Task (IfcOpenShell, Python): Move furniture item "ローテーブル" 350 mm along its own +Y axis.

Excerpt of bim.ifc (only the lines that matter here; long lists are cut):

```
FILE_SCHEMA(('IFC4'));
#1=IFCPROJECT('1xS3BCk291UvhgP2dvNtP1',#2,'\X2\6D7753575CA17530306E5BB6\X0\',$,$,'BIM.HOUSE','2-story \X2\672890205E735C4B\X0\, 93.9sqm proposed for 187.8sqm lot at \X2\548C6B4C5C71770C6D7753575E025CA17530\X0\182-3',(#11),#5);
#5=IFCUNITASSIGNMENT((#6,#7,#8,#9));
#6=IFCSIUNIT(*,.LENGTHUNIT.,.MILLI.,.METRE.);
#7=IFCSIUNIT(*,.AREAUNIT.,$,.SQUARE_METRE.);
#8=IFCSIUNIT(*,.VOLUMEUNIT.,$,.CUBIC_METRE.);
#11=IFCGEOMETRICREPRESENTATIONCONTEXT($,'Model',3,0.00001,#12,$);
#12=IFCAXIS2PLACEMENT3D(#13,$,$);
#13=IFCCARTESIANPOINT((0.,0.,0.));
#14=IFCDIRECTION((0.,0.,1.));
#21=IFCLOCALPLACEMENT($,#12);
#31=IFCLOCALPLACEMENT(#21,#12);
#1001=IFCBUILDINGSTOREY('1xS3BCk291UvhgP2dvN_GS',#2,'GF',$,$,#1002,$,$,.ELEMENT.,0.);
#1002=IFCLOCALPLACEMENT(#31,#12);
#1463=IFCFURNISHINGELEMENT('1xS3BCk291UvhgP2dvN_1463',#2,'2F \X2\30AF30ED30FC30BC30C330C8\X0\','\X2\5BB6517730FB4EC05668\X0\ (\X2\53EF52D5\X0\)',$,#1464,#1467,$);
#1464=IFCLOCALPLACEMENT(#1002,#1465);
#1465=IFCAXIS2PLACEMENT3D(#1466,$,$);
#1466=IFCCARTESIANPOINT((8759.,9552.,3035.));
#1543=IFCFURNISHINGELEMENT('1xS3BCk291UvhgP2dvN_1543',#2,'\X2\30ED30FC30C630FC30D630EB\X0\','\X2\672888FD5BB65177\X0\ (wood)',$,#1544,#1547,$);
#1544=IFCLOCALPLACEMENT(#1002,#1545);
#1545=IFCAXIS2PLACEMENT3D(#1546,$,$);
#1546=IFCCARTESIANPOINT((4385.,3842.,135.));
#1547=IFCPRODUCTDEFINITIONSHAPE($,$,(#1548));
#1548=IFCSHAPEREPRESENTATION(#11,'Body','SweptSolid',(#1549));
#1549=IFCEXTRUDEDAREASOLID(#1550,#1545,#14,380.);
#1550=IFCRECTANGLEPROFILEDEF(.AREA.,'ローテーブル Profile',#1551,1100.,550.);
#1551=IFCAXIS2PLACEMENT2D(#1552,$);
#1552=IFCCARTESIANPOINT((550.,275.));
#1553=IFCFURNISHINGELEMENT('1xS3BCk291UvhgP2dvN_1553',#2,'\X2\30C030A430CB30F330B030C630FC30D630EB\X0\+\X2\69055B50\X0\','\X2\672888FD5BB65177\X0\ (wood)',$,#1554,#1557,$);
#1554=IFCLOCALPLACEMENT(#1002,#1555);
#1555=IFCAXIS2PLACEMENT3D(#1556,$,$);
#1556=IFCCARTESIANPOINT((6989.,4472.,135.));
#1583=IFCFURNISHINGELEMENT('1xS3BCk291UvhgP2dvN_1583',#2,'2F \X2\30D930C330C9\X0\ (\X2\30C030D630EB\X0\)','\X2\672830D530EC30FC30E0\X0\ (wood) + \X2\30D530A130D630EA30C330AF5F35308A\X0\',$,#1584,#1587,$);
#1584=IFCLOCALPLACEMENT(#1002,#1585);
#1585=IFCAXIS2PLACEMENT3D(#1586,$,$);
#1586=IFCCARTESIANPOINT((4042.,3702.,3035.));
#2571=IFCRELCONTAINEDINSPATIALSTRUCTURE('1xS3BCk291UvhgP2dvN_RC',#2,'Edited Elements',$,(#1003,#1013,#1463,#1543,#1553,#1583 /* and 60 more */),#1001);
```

```python
import ifcopenshell
import ifcopenshell.api.geometry
import ifcopenshell.util.placement
import ifcopenshell.util.unit

model = ifcopenshell.open("bim.ifc")
unit_scale = ifcopenshell.util.unit.calculate_unit_scale(model)

item = model.by_guid("1xS3BCk291UvhgP2dvN_1543")
matrix = ifcopenshell.util.placement.get_local_placement(item.ObjectPlacement)
matrix[:3, 3] += matrix[:3, 1] * 0.35 / unit_scale
ifcopenshell.api.geometry.edit_object_placement(model, product=item, matrix=matrix, is_si=False)

print(ifcopenshell.util.placement.get_local_placement(item.ObjectPlacement).round(3) + 0.0)

model.write("bim_updated.ifc")
```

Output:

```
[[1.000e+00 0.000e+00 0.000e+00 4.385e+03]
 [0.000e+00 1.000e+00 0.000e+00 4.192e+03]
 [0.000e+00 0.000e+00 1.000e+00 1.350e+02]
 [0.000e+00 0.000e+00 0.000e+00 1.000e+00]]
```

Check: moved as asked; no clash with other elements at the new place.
